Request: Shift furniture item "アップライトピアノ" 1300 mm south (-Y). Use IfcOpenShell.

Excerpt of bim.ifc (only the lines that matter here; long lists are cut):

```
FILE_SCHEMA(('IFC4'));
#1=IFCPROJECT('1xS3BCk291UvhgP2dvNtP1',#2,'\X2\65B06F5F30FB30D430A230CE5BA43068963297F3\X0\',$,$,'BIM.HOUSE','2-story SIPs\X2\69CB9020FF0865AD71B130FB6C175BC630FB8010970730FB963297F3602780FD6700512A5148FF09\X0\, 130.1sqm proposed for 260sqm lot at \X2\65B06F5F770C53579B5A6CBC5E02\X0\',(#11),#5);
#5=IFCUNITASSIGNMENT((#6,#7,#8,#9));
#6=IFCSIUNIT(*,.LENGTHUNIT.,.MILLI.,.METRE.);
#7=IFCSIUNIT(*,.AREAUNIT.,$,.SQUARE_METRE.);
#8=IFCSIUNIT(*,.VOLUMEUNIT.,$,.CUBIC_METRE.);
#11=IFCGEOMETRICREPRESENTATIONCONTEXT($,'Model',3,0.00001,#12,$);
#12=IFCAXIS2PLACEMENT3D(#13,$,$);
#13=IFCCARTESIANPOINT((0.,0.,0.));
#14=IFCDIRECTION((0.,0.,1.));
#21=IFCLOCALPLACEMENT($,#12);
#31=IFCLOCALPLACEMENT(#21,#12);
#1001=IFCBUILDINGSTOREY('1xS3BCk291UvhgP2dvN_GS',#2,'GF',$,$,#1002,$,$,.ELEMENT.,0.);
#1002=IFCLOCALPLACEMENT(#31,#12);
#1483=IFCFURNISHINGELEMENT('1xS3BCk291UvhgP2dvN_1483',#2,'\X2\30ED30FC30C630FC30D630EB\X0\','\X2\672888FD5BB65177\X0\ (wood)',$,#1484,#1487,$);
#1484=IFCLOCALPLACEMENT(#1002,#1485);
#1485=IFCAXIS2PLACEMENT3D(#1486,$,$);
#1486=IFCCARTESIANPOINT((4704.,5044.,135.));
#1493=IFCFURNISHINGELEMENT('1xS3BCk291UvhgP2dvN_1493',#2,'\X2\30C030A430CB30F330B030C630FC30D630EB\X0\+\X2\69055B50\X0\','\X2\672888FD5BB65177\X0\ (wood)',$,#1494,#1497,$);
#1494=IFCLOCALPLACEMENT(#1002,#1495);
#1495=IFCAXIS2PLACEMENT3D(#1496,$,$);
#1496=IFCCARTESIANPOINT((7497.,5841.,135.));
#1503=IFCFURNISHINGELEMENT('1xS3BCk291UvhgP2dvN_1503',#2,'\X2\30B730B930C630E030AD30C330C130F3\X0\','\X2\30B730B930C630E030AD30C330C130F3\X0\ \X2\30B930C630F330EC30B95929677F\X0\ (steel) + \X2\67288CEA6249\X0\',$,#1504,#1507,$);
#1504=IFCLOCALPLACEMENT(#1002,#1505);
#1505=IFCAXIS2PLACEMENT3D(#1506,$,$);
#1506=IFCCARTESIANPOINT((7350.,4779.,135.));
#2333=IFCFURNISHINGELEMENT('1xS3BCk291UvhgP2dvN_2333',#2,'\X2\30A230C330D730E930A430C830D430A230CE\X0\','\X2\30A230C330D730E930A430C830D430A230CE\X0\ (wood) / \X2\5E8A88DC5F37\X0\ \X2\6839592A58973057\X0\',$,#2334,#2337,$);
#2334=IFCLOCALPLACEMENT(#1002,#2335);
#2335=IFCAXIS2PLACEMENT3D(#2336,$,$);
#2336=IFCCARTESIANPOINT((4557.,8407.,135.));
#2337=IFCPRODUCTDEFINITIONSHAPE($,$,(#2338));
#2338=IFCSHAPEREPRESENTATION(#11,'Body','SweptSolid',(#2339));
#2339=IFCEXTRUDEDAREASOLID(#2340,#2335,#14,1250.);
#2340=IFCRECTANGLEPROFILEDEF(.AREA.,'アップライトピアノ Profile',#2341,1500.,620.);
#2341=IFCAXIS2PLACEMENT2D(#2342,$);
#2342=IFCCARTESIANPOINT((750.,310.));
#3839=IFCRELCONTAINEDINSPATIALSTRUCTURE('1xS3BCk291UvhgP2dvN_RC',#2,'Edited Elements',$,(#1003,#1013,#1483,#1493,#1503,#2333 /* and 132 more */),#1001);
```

```python
import ifcopenshell
import ifcopenshell.api.geometry
import ifcopenshell.util.placement

model = ifcopenshell.open("bim.ifc")

item = model.by_guid("1xS3BCk291UvhgP2dvN_2333")
matrix = ifcopenshell.util.placement.get_local_placement(item.ObjectPlacement)
matrix[1, 3] -= 1300.0
ifcopenshell.api.geometry.edit_object_placement(model, product=item, matrix=matrix, is_si=False)

print(ifcopenshell.util.placement.get_local_placement(item.ObjectPlacement).round(3) + 0.0)

model.write("bim-out.ifc")
```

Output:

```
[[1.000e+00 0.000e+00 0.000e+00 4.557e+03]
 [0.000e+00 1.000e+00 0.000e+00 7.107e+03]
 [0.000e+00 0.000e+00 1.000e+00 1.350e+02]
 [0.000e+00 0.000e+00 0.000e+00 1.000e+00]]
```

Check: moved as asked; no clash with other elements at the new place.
